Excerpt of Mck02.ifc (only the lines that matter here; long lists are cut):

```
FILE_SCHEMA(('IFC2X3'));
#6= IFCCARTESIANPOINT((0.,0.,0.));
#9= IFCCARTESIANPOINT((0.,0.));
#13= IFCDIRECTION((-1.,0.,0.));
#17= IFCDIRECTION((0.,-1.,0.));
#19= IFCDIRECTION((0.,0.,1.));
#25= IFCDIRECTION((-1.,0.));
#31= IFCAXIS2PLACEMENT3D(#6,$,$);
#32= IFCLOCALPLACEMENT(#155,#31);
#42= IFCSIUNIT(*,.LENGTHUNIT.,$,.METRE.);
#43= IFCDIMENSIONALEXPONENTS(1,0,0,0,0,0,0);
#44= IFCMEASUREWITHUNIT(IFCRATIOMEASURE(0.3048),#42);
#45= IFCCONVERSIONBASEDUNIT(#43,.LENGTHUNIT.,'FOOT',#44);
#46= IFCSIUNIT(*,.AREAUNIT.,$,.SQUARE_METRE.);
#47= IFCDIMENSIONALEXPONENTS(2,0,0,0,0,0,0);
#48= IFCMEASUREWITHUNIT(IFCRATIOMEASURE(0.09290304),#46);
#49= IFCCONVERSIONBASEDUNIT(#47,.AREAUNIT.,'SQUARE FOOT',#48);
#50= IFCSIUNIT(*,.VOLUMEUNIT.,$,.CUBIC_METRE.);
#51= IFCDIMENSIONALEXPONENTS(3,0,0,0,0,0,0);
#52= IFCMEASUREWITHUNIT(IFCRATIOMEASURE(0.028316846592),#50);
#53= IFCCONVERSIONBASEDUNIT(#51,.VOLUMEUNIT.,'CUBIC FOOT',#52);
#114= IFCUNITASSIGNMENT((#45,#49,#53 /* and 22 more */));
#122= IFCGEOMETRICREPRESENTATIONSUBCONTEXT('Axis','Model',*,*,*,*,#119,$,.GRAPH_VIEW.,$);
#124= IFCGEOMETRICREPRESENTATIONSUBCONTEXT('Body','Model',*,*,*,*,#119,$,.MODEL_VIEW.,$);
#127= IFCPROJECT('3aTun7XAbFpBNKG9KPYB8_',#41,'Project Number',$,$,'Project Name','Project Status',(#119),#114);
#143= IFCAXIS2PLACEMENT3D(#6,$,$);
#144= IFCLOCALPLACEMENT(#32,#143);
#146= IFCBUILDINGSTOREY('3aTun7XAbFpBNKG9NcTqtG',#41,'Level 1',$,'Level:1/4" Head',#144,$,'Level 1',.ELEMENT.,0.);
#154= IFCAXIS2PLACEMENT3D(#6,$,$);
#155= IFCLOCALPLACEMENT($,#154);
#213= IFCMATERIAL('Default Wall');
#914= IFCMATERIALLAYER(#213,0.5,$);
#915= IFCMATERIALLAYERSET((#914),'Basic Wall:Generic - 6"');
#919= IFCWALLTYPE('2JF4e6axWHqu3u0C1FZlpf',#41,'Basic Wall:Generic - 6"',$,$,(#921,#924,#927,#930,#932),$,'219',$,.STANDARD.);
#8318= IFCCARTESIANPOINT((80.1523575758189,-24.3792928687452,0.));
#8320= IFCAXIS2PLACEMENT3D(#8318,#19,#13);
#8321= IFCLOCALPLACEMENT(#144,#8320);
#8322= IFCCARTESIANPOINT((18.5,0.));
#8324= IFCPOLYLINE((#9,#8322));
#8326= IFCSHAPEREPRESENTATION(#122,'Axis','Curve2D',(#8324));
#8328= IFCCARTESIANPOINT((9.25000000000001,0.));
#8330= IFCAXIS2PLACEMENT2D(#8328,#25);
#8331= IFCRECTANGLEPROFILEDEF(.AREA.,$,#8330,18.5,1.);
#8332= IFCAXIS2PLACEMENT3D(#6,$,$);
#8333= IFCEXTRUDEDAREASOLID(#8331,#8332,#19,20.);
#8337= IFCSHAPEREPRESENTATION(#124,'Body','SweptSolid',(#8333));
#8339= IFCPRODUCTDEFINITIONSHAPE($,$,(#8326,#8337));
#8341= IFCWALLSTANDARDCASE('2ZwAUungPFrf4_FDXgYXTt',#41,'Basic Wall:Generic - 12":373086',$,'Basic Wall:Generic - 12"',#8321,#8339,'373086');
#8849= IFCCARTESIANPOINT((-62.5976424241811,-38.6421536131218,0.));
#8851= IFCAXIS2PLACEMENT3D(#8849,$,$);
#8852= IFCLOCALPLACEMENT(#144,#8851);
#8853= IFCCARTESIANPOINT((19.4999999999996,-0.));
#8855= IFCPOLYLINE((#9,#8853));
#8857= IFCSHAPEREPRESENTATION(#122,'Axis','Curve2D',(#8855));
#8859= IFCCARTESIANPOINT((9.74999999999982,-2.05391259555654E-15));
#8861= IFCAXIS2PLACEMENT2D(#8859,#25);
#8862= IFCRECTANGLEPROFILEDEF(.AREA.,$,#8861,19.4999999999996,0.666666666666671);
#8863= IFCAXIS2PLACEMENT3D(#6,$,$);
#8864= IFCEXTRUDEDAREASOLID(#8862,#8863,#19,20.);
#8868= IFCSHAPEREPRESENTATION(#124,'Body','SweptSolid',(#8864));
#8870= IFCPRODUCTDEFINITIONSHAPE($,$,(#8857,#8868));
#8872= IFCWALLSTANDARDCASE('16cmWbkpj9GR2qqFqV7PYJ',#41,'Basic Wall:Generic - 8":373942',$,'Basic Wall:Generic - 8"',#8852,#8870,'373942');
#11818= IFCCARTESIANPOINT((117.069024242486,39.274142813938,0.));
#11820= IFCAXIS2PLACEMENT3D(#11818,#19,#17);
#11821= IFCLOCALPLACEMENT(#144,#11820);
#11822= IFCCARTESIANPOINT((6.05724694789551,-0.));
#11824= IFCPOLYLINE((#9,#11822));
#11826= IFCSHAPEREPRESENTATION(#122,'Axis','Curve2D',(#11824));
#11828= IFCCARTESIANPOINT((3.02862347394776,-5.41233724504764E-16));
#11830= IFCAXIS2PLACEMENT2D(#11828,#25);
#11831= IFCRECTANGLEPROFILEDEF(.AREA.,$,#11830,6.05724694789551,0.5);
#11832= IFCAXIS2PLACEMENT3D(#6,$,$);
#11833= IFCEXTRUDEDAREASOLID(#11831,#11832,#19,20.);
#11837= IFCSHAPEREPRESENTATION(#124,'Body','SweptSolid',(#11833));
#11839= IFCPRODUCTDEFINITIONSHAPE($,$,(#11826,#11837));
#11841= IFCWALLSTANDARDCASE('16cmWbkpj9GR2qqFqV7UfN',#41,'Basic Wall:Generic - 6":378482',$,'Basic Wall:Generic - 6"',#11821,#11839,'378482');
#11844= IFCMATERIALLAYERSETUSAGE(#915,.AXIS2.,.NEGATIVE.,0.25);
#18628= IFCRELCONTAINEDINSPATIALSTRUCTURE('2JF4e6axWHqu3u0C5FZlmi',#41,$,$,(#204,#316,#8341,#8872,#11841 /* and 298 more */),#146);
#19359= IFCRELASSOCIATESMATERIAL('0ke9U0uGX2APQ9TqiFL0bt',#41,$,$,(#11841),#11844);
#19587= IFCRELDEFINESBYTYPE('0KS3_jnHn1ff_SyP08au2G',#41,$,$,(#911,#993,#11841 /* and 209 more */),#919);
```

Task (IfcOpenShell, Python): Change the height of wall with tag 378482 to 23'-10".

```python
import ifcopenshell
import ifcopenshell.geom
import ifcopenshell.util.representation
import ifcopenshell.util.shape
import ifcopenshell.util.unit

model = ifcopenshell.open("Mck02.ifc")
unit_scale = ifcopenshell.util.unit.calculate_unit_scale(model)
settings = ifcopenshell.geom.settings()


def volume(element):
    """Net volume in cubic metres, openings subtracted."""
    shape = ifcopenshell.geom.create_shape(settings, element)
    return ifcopenshell.util.shape.get_volume(shape.geometry)


wall = model.by_guid("16cmWbkpj9GR2qqFqV7UfN")
before = volume(wall)

body = ifcopenshell.util.representation.get_representation(wall, "Model", "Body")
solid = body.Items[0]
old_height = solid.Depth
solid.Depth = 286 * 0.0254 / unit_scale
after = volume(wall)

print(f"height {old_height:g} -> {solid.Depth:g}, volume {before:.3f} -> {after:.3f} m3")

model.write("Mck02_edited.ifc")
```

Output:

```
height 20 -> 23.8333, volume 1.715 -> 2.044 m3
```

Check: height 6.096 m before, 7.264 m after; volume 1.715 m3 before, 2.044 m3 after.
